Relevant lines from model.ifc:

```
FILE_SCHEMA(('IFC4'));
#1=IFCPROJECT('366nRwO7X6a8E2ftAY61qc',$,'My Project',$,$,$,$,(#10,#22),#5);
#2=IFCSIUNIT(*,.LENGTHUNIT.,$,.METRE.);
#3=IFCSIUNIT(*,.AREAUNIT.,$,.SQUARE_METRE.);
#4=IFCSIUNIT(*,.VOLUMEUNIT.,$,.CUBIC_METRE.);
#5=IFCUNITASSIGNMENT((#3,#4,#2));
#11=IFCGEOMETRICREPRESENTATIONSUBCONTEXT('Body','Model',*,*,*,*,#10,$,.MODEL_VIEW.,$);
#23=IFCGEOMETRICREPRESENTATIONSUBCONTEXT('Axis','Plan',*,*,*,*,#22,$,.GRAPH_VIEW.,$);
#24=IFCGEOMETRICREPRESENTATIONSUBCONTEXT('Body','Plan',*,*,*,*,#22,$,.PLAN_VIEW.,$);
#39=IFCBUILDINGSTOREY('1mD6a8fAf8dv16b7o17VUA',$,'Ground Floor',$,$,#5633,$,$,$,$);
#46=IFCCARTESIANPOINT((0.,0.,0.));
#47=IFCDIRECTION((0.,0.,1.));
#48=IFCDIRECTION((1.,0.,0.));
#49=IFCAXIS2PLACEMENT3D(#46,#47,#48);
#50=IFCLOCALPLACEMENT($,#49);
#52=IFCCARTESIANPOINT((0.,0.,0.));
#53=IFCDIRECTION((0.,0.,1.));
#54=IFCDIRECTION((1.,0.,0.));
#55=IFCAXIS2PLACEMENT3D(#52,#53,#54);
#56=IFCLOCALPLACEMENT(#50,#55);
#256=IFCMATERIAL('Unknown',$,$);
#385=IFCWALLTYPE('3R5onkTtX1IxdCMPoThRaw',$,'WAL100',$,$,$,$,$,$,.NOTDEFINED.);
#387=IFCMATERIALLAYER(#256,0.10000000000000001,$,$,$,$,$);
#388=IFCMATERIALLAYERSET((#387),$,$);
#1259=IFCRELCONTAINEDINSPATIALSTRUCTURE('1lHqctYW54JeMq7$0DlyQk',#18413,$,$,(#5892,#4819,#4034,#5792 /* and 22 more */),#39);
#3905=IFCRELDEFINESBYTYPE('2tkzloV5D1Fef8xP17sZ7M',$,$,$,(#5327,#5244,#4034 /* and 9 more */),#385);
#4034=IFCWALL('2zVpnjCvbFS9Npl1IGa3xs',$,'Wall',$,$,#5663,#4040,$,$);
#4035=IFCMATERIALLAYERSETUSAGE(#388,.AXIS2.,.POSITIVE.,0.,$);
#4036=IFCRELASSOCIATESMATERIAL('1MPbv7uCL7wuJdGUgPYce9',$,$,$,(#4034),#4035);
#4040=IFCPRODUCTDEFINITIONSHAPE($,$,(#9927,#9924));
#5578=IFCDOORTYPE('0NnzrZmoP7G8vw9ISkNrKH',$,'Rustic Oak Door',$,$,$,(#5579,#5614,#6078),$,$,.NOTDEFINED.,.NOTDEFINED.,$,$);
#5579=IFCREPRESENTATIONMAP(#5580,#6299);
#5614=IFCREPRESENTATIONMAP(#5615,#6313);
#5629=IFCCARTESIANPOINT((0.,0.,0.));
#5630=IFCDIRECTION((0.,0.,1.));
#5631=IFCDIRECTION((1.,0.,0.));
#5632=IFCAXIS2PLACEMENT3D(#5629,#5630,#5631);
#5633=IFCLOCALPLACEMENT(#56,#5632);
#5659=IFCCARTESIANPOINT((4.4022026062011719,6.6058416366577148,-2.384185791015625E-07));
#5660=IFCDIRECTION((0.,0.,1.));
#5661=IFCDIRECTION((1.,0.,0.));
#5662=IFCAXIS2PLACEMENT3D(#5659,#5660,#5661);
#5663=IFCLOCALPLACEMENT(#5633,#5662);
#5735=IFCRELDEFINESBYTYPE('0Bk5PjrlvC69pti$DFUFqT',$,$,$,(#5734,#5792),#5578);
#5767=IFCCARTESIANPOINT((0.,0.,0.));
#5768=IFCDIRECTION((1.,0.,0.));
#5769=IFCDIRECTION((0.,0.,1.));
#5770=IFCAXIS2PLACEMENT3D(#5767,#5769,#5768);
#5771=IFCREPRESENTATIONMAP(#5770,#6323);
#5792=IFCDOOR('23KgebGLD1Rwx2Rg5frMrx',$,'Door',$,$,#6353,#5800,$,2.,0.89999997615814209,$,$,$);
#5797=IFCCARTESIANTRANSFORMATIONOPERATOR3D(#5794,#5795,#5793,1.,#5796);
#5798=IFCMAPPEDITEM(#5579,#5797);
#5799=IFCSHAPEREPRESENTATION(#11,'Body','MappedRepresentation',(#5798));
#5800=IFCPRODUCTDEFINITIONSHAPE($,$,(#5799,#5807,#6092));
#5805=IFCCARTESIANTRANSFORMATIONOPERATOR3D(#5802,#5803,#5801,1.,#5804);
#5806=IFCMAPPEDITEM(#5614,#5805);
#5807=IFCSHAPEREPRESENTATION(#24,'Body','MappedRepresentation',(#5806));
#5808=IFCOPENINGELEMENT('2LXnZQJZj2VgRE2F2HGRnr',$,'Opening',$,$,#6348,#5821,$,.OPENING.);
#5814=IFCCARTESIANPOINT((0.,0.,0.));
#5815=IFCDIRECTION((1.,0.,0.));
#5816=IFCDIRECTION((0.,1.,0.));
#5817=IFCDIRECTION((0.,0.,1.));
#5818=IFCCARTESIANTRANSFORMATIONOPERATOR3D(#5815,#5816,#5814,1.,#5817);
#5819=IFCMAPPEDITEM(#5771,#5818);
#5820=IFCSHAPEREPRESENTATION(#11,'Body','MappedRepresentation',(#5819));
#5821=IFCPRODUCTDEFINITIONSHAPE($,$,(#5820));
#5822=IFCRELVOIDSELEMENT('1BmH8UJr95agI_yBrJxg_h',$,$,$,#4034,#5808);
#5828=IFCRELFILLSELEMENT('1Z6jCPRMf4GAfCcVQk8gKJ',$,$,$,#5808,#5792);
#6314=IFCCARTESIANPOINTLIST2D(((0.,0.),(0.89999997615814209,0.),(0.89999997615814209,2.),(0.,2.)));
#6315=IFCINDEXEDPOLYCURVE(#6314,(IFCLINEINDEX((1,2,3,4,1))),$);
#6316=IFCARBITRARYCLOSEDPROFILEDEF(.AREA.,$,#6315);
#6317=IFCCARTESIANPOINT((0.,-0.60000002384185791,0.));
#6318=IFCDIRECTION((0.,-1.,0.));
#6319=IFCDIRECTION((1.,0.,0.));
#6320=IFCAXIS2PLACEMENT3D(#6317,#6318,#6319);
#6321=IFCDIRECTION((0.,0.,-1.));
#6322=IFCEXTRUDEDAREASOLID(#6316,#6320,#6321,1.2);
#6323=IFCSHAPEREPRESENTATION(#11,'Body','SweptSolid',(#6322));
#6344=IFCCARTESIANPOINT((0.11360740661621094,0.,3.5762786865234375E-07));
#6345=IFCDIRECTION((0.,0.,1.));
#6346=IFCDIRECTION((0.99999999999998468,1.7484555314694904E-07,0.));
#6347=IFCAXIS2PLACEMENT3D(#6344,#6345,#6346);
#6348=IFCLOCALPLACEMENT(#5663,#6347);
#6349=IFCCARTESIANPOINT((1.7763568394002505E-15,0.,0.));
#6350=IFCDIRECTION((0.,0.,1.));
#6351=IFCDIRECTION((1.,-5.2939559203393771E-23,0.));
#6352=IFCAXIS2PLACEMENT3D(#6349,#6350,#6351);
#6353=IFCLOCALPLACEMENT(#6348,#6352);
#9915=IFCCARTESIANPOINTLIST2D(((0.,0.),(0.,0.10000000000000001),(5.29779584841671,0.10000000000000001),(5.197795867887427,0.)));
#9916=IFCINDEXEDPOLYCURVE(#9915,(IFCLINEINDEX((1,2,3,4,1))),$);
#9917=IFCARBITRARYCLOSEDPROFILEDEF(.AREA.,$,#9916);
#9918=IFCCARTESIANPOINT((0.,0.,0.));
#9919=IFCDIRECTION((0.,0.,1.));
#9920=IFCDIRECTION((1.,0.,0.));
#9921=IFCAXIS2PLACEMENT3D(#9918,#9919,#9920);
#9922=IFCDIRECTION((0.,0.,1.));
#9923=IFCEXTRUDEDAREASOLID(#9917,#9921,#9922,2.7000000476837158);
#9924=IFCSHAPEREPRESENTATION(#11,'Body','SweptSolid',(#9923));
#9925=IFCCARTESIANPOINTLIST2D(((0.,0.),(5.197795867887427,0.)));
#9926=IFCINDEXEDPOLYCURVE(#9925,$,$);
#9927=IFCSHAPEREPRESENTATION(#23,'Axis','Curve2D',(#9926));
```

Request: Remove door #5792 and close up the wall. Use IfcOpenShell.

```python
import ifcopenshell
import ifcopenshell.api.feature
import ifcopenshell.api.root
import ifcopenshell.geom
import ifcopenshell.util.shape

model = ifcopenshell.open("model.ifc")
settings = ifcopenshell.geom.settings()


def volume(element):
    """Net volume in cubic metres, openings subtracted."""
    shape = ifcopenshell.geom.create_shape(settings, element)
    return ifcopenshell.util.shape.get_volume(shape.geometry)


door = model.by_guid("23KgebGLD1Rwx2Rg5frMrx")
opening = door.FillsVoids[0].RelatingOpeningElement
wall = opening.VoidsElements[0].RelatingBuildingElement
before = volume(wall)

ifcopenshell.api.root.remove_product(model, product=door)
ifcopenshell.api.feature.remove_feature(model, feature=opening)

after = volume(wall)

print(f"wall volume {before:.3f} -> {after:.3f} m3")

model.write("model-out.ifc")
```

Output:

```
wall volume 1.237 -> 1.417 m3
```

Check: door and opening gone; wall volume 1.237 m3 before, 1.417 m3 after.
